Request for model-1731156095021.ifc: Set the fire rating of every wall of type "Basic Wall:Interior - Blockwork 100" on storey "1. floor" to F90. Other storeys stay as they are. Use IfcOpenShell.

First a look at what the model holds.

```python
import ifcopenshell
import ifcopenshell.util.element

model = ifcopenshell.open("model-1731156095021.ifc")
print(model.schema)
storey = next(s for s in model.by_type("IfcBuildingStorey") if s.Name == "1. floor")
walls = [e for e in ifcopenshell.util.element.get_decomposition(storey) if e.is_a("IfcWall")]
seen = {}
for e in walls:
    element_type = ifcopenshell.util.element.get_type(e)
    key = (element_type.Name if element_type != e and element_type else None, ifcopenshell.util.element.get_pset(e, "Pset_WallCommon", "FireRating"))
    seen[key] = seen.get(key, 0) + 1
for (name, value), count in sorted(seen.items(), key=str):
    print(count, "x", name, "|", value)
```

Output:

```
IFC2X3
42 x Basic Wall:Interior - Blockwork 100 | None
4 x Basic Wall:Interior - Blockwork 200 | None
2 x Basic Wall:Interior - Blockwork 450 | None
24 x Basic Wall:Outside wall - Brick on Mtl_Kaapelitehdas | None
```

```python
import ifcopenshell
import ifcopenshell.api.pset
import ifcopenshell.util.element

model = ifcopenshell.open("model-1731156095021.ifc")

storey = next(s for s in model.by_type("IfcBuildingStorey") if s.Name == "1. floor")
walls = [e for e in ifcopenshell.util.element.get_decomposition(storey) if e.is_a("IfcWall")]

count = 0
for e in walls:
    element_type = ifcopenshell.util.element.get_type(e)
    if element_type in (None, e) or element_type.Name != "Basic Wall:Interior - Blockwork 100":
        continue
    # add_pset returns the element's existing set when there is one.
    pset = ifcopenshell.api.pset.add_pset(model, product=e, name="Pset_WallCommon")
    ifcopenshell.api.pset.edit_pset(model, pset=pset, properties={"FireRating": "F90"})
    count += 1

print(count, "walls updated")

model.write("model-1731156095021_rev.ifc")
```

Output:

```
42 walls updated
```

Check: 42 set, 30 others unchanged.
